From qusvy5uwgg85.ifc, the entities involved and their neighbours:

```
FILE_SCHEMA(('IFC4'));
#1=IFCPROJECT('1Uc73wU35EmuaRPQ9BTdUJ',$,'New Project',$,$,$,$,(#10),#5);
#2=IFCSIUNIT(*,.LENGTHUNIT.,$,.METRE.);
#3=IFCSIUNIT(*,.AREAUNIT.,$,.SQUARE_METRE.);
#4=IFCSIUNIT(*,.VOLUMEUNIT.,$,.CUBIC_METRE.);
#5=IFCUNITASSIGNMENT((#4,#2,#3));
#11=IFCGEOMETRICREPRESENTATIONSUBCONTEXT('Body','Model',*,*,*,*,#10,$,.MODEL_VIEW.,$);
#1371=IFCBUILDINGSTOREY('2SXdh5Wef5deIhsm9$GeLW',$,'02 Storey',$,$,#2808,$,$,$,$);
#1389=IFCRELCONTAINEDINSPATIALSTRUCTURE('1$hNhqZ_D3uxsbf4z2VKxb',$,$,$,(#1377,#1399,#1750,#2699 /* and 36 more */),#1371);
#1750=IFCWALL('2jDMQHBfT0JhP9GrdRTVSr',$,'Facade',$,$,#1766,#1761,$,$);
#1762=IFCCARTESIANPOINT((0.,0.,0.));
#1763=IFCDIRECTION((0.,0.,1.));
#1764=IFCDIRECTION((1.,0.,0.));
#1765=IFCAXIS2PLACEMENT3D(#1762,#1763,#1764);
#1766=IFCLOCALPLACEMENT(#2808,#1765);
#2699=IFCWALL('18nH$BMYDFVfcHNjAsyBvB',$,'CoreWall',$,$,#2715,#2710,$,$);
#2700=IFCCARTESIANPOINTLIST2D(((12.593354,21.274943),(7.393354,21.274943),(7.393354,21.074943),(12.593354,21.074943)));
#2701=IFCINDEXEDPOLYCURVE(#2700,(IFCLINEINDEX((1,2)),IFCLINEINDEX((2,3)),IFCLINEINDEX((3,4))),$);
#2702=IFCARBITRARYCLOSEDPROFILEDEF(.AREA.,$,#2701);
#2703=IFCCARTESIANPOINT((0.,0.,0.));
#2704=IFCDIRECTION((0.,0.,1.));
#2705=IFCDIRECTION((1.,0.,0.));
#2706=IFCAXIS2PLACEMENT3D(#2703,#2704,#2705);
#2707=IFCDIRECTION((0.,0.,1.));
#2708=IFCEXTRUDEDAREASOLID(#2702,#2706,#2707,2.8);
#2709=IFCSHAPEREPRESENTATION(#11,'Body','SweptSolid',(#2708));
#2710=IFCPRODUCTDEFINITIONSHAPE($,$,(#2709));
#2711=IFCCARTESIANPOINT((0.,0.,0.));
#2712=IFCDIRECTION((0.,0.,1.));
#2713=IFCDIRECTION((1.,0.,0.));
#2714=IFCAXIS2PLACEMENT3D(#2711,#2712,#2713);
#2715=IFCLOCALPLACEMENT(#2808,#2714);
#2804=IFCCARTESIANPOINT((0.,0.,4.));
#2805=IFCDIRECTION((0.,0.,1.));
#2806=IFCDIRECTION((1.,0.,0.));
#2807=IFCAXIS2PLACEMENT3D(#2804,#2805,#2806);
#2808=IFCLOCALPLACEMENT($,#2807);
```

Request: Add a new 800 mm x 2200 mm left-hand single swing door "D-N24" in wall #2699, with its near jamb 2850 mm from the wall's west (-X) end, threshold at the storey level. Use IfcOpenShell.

```python
import numpy as np
import ifcopenshell
import ifcopenshell.api.feature
import ifcopenshell.api.geometry
import ifcopenshell.api.root
import ifcopenshell.api.spatial
import ifcopenshell.geom
import ifcopenshell.util.element
import ifcopenshell.util.placement
import ifcopenshell.util.representation
import ifcopenshell.util.shape
import ifcopenshell.util.unit

model = ifcopenshell.open("qusvy5uwgg85.ifc")
unit_scale = ifcopenshell.util.unit.calculate_unit_scale(model)
settings = ifcopenshell.geom.settings()


def volume(element):
    """Net volume in cubic metres, openings subtracted."""
    shape = ifcopenshell.geom.create_shape(settings, element)
    return ifcopenshell.util.shape.get_volume(shape.geometry)


wall = model.by_guid("18nH$BMYDFVfcHNjAsyBvB")
storey = ifcopenshell.util.element.get_container(wall, ifc_class="IfcBuildingStorey")
context = ifcopenshell.util.representation.get_context(model, "Model", "Body", "MODEL_VIEW")
before = volume(wall)

width, height, from_end, sill = 0.8, 2.2, 2.85, 0.0  # metres

# The wall runs along its own X axis, and the end named is its -X end.
wall_shape = ifcopenshell.geom.create_shape(settings, wall)
x, y, z = ifcopenshell.util.shape.get_vertices(wall_shape.geometry).T
start = x.min() + from_end
face, thickness = float(y.min()), float(y.max() - y.min())
wall_matrix = ifcopenshell.util.placement.get_local_placement(wall.ObjectPlacement)
level = ifcopenshell.util.placement.get_local_placement(storey.ObjectPlacement)[2, 3]


def in_wall(x, y):
    """Placement at x, y metres in the wall's axes, at sill height."""
    matrix = wall_matrix.copy()
    matrix[:, 3] = wall_matrix @ np.array([x / unit_scale, y / unit_scale, 0.0, 1.0])
    matrix[2, 3] = level + sill / unit_scale
    return matrix


# Opening: a box that overshoots both wall faces by 50 mm.
opening = ifcopenshell.api.root.create_entity(model, ifc_class="IfcOpeningElement", predefined_type="OPENING")
box = ifcopenshell.api.geometry.add_wall_representation(
    model, context=context, length=width, height=height, thickness=thickness + 0.1
)
ifcopenshell.api.geometry.assign_representation(model, product=opening, representation=box)
ifcopenshell.api.geometry.edit_object_placement(model, product=opening, matrix=in_wall(start, face - 0.05), is_si=False)
ifcopenshell.api.feature.add_feature(model, feature=opening, element=wall)

door = ifcopenshell.api.root.create_entity(model, ifc_class="IfcDoor", name="D-N24", predefined_type="DOOR")
door.OverallWidth, door.OverallHeight = width / unit_scale, height / unit_scale
door.OperationType = "SINGLE_SWING_LEFT"
body = ifcopenshell.api.geometry.add_door_representation(
    model,
    context=context,
    overall_width=door.OverallWidth,
    overall_height=door.OverallHeight,
    operation_type="SINGLE_SWING_LEFT",
    lining_properties={"LiningDepth": thickness / unit_scale, "ThresholdDepth": thickness / unit_scale},
)
ifcopenshell.api.geometry.assign_representation(model, product=door, representation=body)
ifcopenshell.api.spatial.assign_container(model, products=[door], relating_structure=storey)
ifcopenshell.api.feature.add_filling(model, opening=opening, element=door)

# The lining spans the wall, so the door starts at the wall face.
ifcopenshell.api.geometry.edit_object_placement(model, product=door, matrix=in_wall(start, face), is_si=False)

after = volume(wall)

print(f"wall volume {before:.3f} -> {after:.3f} m3")

model.write("qusvy5uwgg85_edited.ifc")
```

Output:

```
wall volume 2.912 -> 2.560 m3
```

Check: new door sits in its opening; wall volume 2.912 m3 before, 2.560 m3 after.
